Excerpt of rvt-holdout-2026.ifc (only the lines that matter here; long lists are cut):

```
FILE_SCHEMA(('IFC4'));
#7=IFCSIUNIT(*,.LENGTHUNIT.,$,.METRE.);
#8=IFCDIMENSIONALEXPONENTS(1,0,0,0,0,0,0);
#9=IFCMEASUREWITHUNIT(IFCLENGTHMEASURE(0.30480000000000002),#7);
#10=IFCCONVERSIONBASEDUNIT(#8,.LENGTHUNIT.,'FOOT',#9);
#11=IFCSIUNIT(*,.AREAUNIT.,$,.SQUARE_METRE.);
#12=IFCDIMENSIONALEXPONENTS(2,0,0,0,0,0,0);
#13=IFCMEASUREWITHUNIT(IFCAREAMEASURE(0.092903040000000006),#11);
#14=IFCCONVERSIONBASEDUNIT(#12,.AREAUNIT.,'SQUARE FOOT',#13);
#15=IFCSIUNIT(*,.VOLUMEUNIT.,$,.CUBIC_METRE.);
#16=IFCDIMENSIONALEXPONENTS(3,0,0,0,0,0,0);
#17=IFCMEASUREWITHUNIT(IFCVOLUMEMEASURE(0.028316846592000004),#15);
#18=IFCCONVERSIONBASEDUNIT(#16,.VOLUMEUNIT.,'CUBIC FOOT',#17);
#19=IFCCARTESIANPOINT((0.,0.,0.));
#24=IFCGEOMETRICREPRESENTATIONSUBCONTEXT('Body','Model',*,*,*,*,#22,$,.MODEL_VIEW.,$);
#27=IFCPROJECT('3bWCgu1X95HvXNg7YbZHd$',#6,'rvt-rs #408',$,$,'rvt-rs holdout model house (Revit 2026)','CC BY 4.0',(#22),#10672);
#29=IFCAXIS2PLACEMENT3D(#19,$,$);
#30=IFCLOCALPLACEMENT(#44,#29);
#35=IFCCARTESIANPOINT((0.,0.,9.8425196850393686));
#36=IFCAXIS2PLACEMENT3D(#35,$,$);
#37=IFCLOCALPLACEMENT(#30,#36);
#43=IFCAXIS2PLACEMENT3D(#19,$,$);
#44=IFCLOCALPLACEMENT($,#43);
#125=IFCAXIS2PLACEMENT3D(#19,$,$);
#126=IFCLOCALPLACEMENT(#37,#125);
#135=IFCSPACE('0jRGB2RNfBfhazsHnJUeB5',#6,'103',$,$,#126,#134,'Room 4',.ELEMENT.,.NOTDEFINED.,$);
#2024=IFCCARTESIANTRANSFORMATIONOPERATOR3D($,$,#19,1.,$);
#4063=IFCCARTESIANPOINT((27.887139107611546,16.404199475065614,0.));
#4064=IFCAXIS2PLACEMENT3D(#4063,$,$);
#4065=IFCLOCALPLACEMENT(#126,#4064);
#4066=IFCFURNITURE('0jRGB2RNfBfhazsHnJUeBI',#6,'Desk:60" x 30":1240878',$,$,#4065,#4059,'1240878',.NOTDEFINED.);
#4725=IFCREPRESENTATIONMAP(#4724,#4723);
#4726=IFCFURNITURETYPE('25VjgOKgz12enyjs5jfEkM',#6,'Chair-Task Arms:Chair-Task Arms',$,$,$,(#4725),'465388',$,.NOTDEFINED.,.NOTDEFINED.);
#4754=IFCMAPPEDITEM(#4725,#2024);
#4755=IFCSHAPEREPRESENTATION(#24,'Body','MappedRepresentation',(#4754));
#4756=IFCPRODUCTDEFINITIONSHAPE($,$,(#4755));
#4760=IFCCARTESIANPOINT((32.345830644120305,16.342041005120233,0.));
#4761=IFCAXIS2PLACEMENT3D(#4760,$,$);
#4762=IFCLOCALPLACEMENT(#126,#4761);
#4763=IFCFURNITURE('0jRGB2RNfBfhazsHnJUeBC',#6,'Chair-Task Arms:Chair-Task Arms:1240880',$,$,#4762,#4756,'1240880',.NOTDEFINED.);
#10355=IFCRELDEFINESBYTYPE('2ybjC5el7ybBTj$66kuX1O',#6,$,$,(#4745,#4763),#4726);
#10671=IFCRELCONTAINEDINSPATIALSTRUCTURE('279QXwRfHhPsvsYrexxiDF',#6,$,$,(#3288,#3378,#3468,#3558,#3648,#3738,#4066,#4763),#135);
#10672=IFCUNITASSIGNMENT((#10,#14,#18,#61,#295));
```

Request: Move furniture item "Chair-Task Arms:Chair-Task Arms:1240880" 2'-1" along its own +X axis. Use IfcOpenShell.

```python
import ifcopenshell
import ifcopenshell.api.geometry
import ifcopenshell.util.placement
import ifcopenshell.util.unit

model = ifcopenshell.open("rvt-holdout-2026.ifc")
unit_scale = ifcopenshell.util.unit.calculate_unit_scale(model)

item = model.by_guid("0jRGB2RNfBfhazsHnJUeBC")
matrix = ifcopenshell.util.placement.get_local_placement(item.ObjectPlacement)
matrix[:3, 3] += matrix[:3, 0] * 25 * 0.0254 / unit_scale
ifcopenshell.api.geometry.edit_object_placement(model, product=item, matrix=matrix, is_si=False)

print(ifcopenshell.util.placement.get_local_placement(item.ObjectPlacement).round(3) + 0.0)

model.write("rvt-holdout-2026_edited.ifc")
```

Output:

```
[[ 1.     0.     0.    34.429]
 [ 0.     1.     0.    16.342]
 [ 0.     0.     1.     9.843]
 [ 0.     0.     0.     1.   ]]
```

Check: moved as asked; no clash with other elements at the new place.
